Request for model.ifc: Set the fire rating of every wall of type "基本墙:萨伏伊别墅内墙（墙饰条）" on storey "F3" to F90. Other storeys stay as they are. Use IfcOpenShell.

First a look at what the model holds.

```python
import ifcopenshell
import ifcopenshell.util.element

model = ifcopenshell.open("model.ifc")
print(model.schema)
storey = next(s for s in model.by_type("IfcBuildingStorey") if s.Name == "F3")
walls = [e for e in ifcopenshell.util.element.get_decomposition(storey) if e.is_a("IfcWall")]
seen = {}
for e in walls:
    element_type = ifcopenshell.util.element.get_type(e)
    key = (element_type.Name if element_type != e and element_type else None, ifcopenshell.util.element.get_pset(e, "Pset_WallCommon", "FireRating"))
    seen[key] = seen.get(key, 0) + 1
for (name, value), count in sorted(seen.items(), key=str):
    print(count, "x", name, "|", value)
```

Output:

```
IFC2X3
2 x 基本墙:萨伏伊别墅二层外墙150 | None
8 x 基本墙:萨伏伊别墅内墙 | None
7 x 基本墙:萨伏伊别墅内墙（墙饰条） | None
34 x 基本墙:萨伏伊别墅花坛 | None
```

```python
import ifcopenshell
import ifcopenshell.api.pset
import ifcopenshell.util.element

model = ifcopenshell.open("model.ifc")

storey = next(s for s in model.by_type("IfcBuildingStorey") if s.Name == "F3")
walls = [e for e in ifcopenshell.util.element.get_decomposition(storey) if e.is_a("IfcWall")]

count = 0
for e in walls:
    element_type = ifcopenshell.util.element.get_type(e)
    if element_type in (None, e) or element_type.Name != "基本墙:萨伏伊别墅内墙（墙饰条）":
        continue
    # add_pset returns the element's existing set when there is one.
    pset = ifcopenshell.api.pset.add_pset(model, product=e, name="Pset_WallCommon")
    ifcopenshell.api.pset.edit_pset(model, pset=pset, properties={"FireRating": "F90"})
    count += 1

print(count, "walls updated")

model.write("model_v2.ifc")
```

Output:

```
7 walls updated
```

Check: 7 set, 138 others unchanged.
